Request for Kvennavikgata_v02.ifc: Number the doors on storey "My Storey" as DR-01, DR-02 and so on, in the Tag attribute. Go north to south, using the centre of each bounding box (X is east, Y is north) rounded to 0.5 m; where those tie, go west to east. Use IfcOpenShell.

First a look at what the model holds.

```python
import ifcopenshell
import ifcopenshell.util.element
import ifcopenshell.util.placement

model = ifcopenshell.open("Kvennavikgata_v02.ifc")
print(model.schema)
storey = next(s for s in model.by_type("IfcBuildingStorey") if s.Name == "My Storey")
doors = [e for e in ifcopenshell.util.element.get_decomposition(storey) if e.is_a("IfcDoor")]
for e in sorted(doors, key=lambda e: e.id()):
    origin = ifcopenshell.util.placement.get_local_placement(e.ObjectPlacement)[:3, 3]
    print(e.id(), e.Tag, e.Name, origin.round(2) + 0.0, sep=" | ")
```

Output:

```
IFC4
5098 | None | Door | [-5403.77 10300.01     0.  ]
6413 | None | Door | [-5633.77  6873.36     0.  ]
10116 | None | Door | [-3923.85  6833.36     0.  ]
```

```python
import ifcopenshell
import ifcopenshell.geom
import ifcopenshell.util.element
import ifcopenshell.util.shape

model = ifcopenshell.open("Kvennavikgata_v02.ifc")
settings = ifcopenshell.geom.settings()
settings.set("use-world-coords", True)


def centre(element):
    shape = ifcopenshell.geom.create_shape(settings, element)
    return ifcopenshell.util.shape.get_bbox_centroid(shape.geometry)


storey = next(s for s in model.by_type("IfcBuildingStorey") if s.Name == "My Storey")
doors = [e for e in ifcopenshell.util.element.get_decomposition(storey) if e.is_a("IfcDoor")]

# Insertion points can sit at a corner or the storey origin, so sort by the geometry (in metres).
centres = {e: centre(e) for e in doors}
doors.sort(key=lambda e: (-round(centres[e][1] / 0.5), centres[e][0]))

for i, e in enumerate(doors, start=1):
    number = f"DR-{i:02d}"
    e.Tag = number
    print(e.id(), number)

model.write("Kvennavikgata_v02_updated.ifc")
```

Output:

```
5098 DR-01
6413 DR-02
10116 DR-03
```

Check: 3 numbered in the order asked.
